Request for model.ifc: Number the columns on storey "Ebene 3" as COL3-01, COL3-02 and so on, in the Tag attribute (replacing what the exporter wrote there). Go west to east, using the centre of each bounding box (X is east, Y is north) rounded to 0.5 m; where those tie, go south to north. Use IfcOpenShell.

First a look at what the model holds.

```python
import ifcopenshell
import ifcopenshell.util.element
import ifcopenshell.util.placement

model = ifcopenshell.open("model.ifc")
print(model.schema)
storey = next(s for s in model.by_type("IfcBuildingStorey") if s.Name == "Ebene 3")
columns = [e for e in ifcopenshell.util.element.get_decomposition(storey) if e.is_a("IfcColumn")]
for e in sorted(columns, key=lambda e: e.id()):
    origin = ifcopenshell.util.placement.get_local_placement(e.ObjectPlacement)[:3, 3]
    print(e.id(), e.Tag, e.Name, origin.round(2) + 0.0, sep=" | ")
```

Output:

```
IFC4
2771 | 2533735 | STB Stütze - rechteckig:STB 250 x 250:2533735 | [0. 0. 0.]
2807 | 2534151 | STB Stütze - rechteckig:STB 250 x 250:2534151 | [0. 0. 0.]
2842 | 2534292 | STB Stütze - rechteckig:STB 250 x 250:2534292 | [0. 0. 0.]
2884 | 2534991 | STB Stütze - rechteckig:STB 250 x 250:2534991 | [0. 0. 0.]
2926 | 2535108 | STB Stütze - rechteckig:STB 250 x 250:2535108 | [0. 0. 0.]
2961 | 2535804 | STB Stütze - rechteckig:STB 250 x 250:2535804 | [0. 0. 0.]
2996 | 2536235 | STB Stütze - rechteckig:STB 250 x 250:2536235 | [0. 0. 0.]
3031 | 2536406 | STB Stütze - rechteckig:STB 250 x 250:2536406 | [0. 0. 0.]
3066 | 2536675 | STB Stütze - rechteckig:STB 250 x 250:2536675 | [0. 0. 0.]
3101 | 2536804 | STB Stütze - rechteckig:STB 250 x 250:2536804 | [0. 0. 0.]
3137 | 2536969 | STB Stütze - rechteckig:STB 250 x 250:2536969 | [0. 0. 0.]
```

```python
import ifcopenshell
import ifcopenshell.geom
import ifcopenshell.util.element
import ifcopenshell.util.shape

model = ifcopenshell.open("model.ifc")
settings = ifcopenshell.geom.settings()
settings.set("use-world-coords", True)


def centre(element):
    shape = ifcopenshell.geom.create_shape(settings, element)
    return ifcopenshell.util.shape.get_bbox_centroid(shape.geometry)


storey = next(s for s in model.by_type("IfcBuildingStorey") if s.Name == "Ebene 3")
columns = [e for e in ifcopenshell.util.element.get_decomposition(storey) if e.is_a("IfcColumn")]

# Insertion points can sit at a corner or the storey origin, so sort by the geometry (in metres).
centres = {e: centre(e) for e in columns}
columns.sort(key=lambda e: (round(centres[e][0] / 0.5), centres[e][1]))

for i, e in enumerate(columns, start=1):
    number = f"COL3-{i:02d}"
    e.Tag = number
    print(e.id(), number)

model.write("model-out.ifc")
```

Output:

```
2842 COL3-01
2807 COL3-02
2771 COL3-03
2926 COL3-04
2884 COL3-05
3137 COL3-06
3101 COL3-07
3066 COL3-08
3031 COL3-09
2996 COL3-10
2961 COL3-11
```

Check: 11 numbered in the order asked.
